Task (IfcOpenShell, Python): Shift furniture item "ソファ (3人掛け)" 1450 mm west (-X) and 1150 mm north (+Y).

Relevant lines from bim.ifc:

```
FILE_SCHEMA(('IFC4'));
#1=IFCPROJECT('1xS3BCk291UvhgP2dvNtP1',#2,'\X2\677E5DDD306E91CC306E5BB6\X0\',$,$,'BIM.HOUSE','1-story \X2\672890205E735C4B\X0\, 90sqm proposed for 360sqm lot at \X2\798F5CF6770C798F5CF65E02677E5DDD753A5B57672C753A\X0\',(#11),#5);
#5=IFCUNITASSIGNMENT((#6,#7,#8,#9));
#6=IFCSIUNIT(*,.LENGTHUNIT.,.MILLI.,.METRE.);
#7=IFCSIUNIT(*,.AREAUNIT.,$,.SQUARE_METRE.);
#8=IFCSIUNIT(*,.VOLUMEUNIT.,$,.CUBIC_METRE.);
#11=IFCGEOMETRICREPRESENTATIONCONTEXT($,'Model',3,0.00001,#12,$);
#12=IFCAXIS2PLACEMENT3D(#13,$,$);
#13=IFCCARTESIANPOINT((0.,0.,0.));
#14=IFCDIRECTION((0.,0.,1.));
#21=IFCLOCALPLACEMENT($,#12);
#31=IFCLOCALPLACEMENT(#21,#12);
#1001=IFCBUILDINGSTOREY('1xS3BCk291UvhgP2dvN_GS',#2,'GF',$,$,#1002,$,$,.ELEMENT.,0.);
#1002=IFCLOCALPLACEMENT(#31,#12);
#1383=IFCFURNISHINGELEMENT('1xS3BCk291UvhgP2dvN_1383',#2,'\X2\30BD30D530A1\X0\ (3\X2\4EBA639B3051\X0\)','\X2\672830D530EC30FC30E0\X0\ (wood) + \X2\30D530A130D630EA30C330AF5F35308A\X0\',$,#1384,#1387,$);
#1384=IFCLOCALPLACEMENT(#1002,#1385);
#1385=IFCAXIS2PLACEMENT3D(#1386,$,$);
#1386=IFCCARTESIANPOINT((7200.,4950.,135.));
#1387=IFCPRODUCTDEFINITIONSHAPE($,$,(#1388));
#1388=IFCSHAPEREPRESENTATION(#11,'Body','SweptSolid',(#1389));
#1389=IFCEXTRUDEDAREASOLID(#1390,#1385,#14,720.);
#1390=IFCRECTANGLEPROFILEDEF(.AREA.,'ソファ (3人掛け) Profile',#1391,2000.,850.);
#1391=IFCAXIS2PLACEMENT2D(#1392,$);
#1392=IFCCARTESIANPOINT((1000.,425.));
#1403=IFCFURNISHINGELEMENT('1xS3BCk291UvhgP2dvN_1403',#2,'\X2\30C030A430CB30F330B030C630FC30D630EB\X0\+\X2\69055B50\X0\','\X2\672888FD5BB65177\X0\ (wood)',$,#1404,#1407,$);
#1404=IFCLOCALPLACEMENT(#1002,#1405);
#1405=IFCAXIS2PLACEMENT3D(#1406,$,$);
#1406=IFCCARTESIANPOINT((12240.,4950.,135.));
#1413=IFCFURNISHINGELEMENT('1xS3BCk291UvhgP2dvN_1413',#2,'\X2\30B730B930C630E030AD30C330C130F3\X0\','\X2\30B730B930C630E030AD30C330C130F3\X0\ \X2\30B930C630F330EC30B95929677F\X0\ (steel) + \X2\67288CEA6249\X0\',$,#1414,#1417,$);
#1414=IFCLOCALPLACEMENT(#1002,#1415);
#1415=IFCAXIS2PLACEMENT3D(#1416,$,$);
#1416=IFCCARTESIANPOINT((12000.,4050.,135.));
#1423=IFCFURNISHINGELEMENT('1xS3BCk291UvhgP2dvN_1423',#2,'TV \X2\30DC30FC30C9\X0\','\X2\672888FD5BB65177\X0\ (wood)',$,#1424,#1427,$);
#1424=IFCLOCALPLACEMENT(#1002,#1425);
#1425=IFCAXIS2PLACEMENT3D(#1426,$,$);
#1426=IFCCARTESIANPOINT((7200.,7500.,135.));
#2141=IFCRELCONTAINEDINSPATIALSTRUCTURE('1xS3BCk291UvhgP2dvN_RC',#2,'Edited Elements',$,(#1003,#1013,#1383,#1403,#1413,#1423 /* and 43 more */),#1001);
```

```python
import ifcopenshell
import ifcopenshell.api.geometry
import ifcopenshell.util.placement
import ifcopenshell.util.unit

model = ifcopenshell.open("bim.ifc")
unit_scale = ifcopenshell.util.unit.calculate_unit_scale(model)

item = model.by_id(1383)
matrix = ifcopenshell.util.placement.get_local_placement(item.ObjectPlacement)
matrix[0, 3] -= 1.45 / unit_scale
matrix[1, 3] += 1.15 / unit_scale
ifcopenshell.api.geometry.edit_object_placement(model, product=item, matrix=matrix, is_si=False)

print(ifcopenshell.util.placement.get_local_placement(item.ObjectPlacement).round(3) + 0.0)

model.write("bim-out.ifc")
```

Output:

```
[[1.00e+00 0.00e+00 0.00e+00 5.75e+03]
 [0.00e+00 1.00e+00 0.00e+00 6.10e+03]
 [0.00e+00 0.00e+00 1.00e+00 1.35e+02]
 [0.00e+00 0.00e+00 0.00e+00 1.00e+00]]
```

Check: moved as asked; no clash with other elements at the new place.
